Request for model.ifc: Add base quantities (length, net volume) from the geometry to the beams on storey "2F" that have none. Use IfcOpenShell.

First a look at what the model holds.

```python
import ifcopenshell
import ifcopenshell.util.element
import ifcopenshell.util.unit

model = ifcopenshell.open("model.ifc")
print(model.schema)
for unit_type in ("LENGTHUNIT", "AREAUNIT", "VOLUMEUNIT"):
    print(unit_type, ifcopenshell.util.unit.calculate_unit_scale(model, unit_type))
storey = next(s for s in model.by_type("IfcBuildingStorey") if s.Name == "2F")
beams = [e for e in ifcopenshell.util.element.get_decomposition(storey) if e.is_a("IfcBeam")]
for e in sorted(beams, key=lambda e: e.id()):
    print(e.id(), e.is_a(), e.Name, list(ifcopenshell.util.element.get_psets(e, qtos_only=True)), sep=" | ")
```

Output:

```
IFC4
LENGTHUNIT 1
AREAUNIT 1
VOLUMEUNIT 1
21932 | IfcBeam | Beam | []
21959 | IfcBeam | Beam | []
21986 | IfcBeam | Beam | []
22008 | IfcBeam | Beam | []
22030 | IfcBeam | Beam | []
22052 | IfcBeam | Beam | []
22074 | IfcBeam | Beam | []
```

```python
import ifcopenshell
import ifcopenshell.api.pset
import ifcopenshell.geom
import ifcopenshell.util.element
import ifcopenshell.util.shape
import ifcopenshell.util.unit

model = ifcopenshell.open("model.ifc")
unit_scale = ifcopenshell.util.unit.calculate_unit_scale(model)
volume_scale = ifcopenshell.util.unit.calculate_unit_scale(model, "VOLUMEUNIT")
settings = ifcopenshell.geom.settings()

storey = next(s for s in model.by_type("IfcBuildingStorey") if s.Name == "2F")
beams = [e for e in ifcopenshell.util.element.get_decomposition(storey) if e.is_a("IfcBeam")]

for e in sorted(beams, key=lambda e: e.id()):
    if ifcopenshell.util.element.get_psets(e, qtos_only=True, should_inherit=False):
        continue
    # Geometry comes back in metres, in the element's own axes.
    shape = ifcopenshell.geom.create_shape(settings, e)
    values = {
        "Length": ifcopenshell.util.shape.get_max_xyz(shape.geometry) / unit_scale,
        "NetVolume": ifcopenshell.util.shape.get_volume(shape.geometry) / volume_scale,
    }
    qto = ifcopenshell.api.pset.add_qto(model, product=e, name="Qto_BeamBaseQuantities")
    ifcopenshell.api.pset.edit_qto(model, qto=qto, properties=values)
    print(e.id(), {k: round(v, 3) for k, v in values.items()})

model.write("model_rev.ifc")
```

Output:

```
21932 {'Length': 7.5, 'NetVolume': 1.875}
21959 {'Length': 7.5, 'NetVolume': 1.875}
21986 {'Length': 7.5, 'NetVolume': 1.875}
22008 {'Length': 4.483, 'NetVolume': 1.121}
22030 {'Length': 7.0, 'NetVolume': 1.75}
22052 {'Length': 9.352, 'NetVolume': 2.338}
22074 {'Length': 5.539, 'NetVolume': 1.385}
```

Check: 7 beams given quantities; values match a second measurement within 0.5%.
